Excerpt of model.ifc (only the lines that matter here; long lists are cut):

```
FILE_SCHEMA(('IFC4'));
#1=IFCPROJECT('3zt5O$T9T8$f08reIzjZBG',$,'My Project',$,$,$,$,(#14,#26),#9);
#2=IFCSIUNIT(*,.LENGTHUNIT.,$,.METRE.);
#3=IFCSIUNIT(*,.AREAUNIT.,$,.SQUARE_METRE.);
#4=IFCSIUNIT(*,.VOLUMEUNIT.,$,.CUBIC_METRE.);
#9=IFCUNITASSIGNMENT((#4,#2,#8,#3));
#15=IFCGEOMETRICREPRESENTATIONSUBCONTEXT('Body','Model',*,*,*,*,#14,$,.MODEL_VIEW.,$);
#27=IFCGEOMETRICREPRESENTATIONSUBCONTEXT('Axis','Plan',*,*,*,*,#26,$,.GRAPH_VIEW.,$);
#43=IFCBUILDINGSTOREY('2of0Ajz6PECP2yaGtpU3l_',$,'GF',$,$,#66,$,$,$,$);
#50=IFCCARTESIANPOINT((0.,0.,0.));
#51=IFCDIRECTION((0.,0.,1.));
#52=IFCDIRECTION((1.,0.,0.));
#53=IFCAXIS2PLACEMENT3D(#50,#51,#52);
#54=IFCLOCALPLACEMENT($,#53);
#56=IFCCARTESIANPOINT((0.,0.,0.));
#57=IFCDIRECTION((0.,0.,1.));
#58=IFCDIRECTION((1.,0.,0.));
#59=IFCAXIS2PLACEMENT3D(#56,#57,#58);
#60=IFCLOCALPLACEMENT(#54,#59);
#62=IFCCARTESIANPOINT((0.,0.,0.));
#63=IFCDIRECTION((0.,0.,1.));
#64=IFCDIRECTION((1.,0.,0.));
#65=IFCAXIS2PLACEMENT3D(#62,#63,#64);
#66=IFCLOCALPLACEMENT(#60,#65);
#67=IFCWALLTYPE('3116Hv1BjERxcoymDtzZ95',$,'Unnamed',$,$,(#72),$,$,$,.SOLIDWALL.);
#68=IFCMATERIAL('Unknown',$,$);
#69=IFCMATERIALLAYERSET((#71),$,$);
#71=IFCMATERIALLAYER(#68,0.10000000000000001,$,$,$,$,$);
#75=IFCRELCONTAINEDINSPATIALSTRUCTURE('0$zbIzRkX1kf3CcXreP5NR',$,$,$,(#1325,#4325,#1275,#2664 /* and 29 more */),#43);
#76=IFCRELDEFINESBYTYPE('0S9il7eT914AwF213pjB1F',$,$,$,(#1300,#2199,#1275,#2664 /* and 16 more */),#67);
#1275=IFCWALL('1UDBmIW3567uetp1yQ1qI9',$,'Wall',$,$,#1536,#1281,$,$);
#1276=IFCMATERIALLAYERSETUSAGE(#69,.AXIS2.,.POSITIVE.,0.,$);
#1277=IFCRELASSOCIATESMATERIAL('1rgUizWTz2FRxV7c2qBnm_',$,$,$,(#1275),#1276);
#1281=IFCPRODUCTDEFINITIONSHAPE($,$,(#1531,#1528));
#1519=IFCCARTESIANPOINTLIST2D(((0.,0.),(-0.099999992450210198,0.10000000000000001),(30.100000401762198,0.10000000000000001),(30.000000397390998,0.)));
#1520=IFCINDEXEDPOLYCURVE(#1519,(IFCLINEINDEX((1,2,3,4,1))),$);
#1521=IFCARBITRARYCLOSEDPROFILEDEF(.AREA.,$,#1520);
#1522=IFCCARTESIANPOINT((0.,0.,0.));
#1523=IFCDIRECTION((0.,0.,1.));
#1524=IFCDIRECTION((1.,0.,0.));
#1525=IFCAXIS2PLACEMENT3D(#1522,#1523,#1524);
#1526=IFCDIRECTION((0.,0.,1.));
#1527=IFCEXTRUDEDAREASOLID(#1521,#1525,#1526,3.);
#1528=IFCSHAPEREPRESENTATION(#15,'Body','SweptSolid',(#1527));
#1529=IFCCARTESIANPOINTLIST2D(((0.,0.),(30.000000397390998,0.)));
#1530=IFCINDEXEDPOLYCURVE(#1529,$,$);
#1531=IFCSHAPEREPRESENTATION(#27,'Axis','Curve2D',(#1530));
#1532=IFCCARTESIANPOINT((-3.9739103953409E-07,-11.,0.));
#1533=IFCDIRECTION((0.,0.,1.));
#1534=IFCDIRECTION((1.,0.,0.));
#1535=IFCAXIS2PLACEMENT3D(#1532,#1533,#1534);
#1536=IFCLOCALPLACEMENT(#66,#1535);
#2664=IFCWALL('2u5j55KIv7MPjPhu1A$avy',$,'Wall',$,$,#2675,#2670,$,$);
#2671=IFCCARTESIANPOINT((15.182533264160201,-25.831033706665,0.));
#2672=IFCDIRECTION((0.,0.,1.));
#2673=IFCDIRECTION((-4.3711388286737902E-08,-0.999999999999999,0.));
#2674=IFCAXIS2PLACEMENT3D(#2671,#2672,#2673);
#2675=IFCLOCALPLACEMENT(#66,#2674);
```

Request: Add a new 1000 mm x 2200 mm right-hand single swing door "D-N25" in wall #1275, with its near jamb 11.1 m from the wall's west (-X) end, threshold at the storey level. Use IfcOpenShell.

```python
import numpy as np
import ifcopenshell
import ifcopenshell.api.feature
import ifcopenshell.api.geometry
import ifcopenshell.api.root
import ifcopenshell.api.spatial
import ifcopenshell.geom
import ifcopenshell.util.element
import ifcopenshell.util.placement
import ifcopenshell.util.representation
import ifcopenshell.util.shape
import ifcopenshell.util.unit

model = ifcopenshell.open("model.ifc")
unit_scale = ifcopenshell.util.unit.calculate_unit_scale(model)
settings = ifcopenshell.geom.settings()


def volume(element):
    """Net volume in cubic metres, openings subtracted."""
    shape = ifcopenshell.geom.create_shape(settings, element)
    return ifcopenshell.util.shape.get_volume(shape.geometry)


wall = model.by_guid("1UDBmIW3567uetp1yQ1qI9")
storey = ifcopenshell.util.element.get_container(wall, ifc_class="IfcBuildingStorey")
context = ifcopenshell.util.representation.get_context(model, "Model", "Body", "MODEL_VIEW")
before = volume(wall)

width, height, from_end, sill = 1, 2.2, 11.1, 0.0  # metres

# The wall runs along its own X axis, and the end named is its -X end.
wall_shape = ifcopenshell.geom.create_shape(settings, wall)
x, y, z = ifcopenshell.util.shape.get_vertices(wall_shape.geometry).T
start = x.min() + from_end
face, thickness = float(y.min()), float(y.max() - y.min())
wall_matrix = ifcopenshell.util.placement.get_local_placement(wall.ObjectPlacement)
level = ifcopenshell.util.placement.get_local_placement(storey.ObjectPlacement)[2, 3]


def in_wall(x, y):
    """Placement at x, y metres in the wall's axes, at sill height."""
    matrix = wall_matrix.copy()
    matrix[:, 3] = wall_matrix @ np.array([x / unit_scale, y / unit_scale, 0.0, 1.0])
    matrix[2, 3] = level + sill / unit_scale
    return matrix


# Opening: a box that overshoots both wall faces by 50 mm.
opening = ifcopenshell.api.root.create_entity(model, ifc_class="IfcOpeningElement", predefined_type="OPENING")
box = ifcopenshell.api.geometry.add_wall_representation(
    model, context=context, length=width, height=height, thickness=thickness + 0.1
)
ifcopenshell.api.geometry.assign_representation(model, product=opening, representation=box)
ifcopenshell.api.geometry.edit_object_placement(model, product=opening, matrix=in_wall(start, face - 0.05), is_si=False)
ifcopenshell.api.feature.add_feature(model, feature=opening, element=wall)

door = ifcopenshell.api.root.create_entity(model, ifc_class="IfcDoor", name="D-N25", predefined_type="DOOR")
door.OverallWidth, door.OverallHeight = width / unit_scale, height / unit_scale
door.OperationType = "SINGLE_SWING_RIGHT"
body = ifcopenshell.api.geometry.add_door_representation(
    model,
    context=context,
    overall_width=door.OverallWidth,
    overall_height=door.OverallHeight,
    operation_type="SINGLE_SWING_RIGHT",
    lining_properties={"LiningDepth": thickness / unit_scale, "ThresholdDepth": thickness / unit_scale},
)
ifcopenshell.api.geometry.assign_representation(model, product=door, representation=body)
ifcopenshell.api.spatial.assign_container(model, products=[door], relating_structure=storey)
ifcopenshell.api.feature.add_filling(model, opening=opening, element=door)

# The lining spans the wall, so the door starts at the wall face.
ifcopenshell.api.geometry.edit_object_placement(model, product=door, matrix=in_wall(start, face), is_si=False)

after = volume(wall)

print(f"wall volume {before:.3f} -> {after:.3f} m3")

model.write("model-out.ifc")
```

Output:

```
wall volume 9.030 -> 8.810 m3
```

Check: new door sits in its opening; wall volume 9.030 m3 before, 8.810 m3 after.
